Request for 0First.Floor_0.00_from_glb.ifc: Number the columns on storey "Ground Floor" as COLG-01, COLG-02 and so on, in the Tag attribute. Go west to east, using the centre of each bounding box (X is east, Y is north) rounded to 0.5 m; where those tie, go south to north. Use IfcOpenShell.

First a look at what the model holds.

```python
import ifcopenshell
import ifcopenshell.util.element
import ifcopenshell.util.placement

model = ifcopenshell.open("0First.Floor_0.00_from_glb.ifc")
print(model.schema)
storey = next(s for s in model.by_type("IfcBuildingStorey") if s.Name == "Ground Floor")
columns = [e for e in ifcopenshell.util.element.get_decomposition(storey) if e.is_a("IfcColumn")]
for e in sorted(columns, key=lambda e: e.id()):
    origin = ifcopenshell.util.placement.get_local_placement(e.ObjectPlacement)[:3, 3]
    print(e.id(), e.Tag, e.Name, origin.round(2) + 0.0, sep=" | ")
```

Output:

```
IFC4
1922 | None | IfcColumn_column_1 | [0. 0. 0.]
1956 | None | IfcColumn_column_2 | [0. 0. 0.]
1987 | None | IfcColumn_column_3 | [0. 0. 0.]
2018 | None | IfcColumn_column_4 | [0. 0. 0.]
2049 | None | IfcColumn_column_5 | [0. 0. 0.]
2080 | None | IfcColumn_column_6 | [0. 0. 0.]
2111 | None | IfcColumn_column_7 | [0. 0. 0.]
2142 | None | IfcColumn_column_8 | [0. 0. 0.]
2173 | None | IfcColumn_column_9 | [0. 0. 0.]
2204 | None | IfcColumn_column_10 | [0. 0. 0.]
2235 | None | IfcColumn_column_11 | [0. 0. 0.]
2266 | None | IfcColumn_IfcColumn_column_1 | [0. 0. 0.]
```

```python
import ifcopenshell
import ifcopenshell.geom
import ifcopenshell.util.element
import ifcopenshell.util.shape

model = ifcopenshell.open("0First.Floor_0.00_from_glb.ifc")
settings = ifcopenshell.geom.settings()
settings.set("use-world-coords", True)


def centre(element):
    shape = ifcopenshell.geom.create_shape(settings, element)
    return ifcopenshell.util.shape.get_bbox_centroid(shape.geometry)


storey = next(s for s in model.by_type("IfcBuildingStorey") if s.Name == "Ground Floor")
columns = [e for e in ifcopenshell.util.element.get_decomposition(storey) if e.is_a("IfcColumn")]

# Insertion points can sit at a corner or the storey origin, so sort by the geometry (in metres).
centres = {e: centre(e) for e in columns}
columns.sort(key=lambda e: (round(centres[e][0] / 0.5), centres[e][1]))

for i, e in enumerate(columns, start=1):
    number = f"COLG-{i:02d}"
    e.Tag = number
    print(e.id(), number)

model.write("0First.Floor_0.00_from_glb_rev.ifc")
```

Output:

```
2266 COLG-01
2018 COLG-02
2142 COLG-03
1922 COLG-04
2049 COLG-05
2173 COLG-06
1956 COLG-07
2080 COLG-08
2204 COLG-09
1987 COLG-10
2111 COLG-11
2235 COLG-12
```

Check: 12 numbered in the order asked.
